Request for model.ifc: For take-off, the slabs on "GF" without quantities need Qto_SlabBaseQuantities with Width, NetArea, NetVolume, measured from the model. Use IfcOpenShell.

First a look at what the model holds.

```python
import ifcopenshell
import ifcopenshell.util.element
import ifcopenshell.util.unit

model = ifcopenshell.open("model.ifc")
print(model.schema)
for unit_type in ("LENGTHUNIT", "AREAUNIT", "VOLUMEUNIT"):
    print(unit_type, ifcopenshell.util.unit.calculate_unit_scale(model, unit_type))
storey = next(s for s in model.by_type("IfcBuildingStorey") if s.Name == "GF")
slabs = [e for e in ifcopenshell.util.element.get_decomposition(storey) if e.is_a("IfcSlab")]
for e in sorted(slabs, key=lambda e: e.id()):
    print(e.id(), e.is_a(), e.Name, list(ifcopenshell.util.element.get_psets(e, qtos_only=True)), sep=" | ")
```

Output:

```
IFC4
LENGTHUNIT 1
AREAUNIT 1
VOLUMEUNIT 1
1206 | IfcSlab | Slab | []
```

```python
import ifcopenshell
import ifcopenshell.api.pset
import ifcopenshell.geom
import ifcopenshell.util.element
import ifcopenshell.util.shape
import ifcopenshell.util.unit

model = ifcopenshell.open("model.ifc")
unit_scale = ifcopenshell.util.unit.calculate_unit_scale(model)
area_scale = ifcopenshell.util.unit.calculate_unit_scale(model, "AREAUNIT")
volume_scale = ifcopenshell.util.unit.calculate_unit_scale(model, "VOLUMEUNIT")
settings = ifcopenshell.geom.settings()

storey = next(s for s in model.by_type("IfcBuildingStorey") if s.Name == "GF")
slabs = [e for e in ifcopenshell.util.element.get_decomposition(storey) if e.is_a("IfcSlab")]

for e in sorted(slabs, key=lambda e: e.id()):
    if ifcopenshell.util.element.get_psets(e, qtos_only=True, should_inherit=False):
        continue
    # Geometry comes back in metres, in the element's own axes.
    shape = ifcopenshell.geom.create_shape(settings, e)
    values = {
        "Width": ifcopenshell.util.shape.get_z(shape.geometry) / unit_scale,
        "NetArea": ifcopenshell.util.shape.get_footprint_area(shape.geometry) / area_scale,
        "NetVolume": ifcopenshell.util.shape.get_volume(shape.geometry) / volume_scale,
    }
    qto = ifcopenshell.api.pset.add_qto(model, product=e, name="Qto_SlabBaseQuantities")
    ifcopenshell.api.pset.edit_qto(model, qto=qto, properties=values)
    print(e.id(), {k: round(v, 3) for k, v in values.items()})

model.write("model_v2.ifc")
```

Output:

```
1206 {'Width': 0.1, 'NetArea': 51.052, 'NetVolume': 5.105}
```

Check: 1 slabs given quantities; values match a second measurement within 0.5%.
